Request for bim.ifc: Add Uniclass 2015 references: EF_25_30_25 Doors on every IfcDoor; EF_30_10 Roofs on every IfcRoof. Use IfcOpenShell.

First a look at what the model holds.

```python
import ifcopenshell

model = ifcopenshell.open("bim.ifc")
print(model.schema)
print("classifications:", [c.Name for c in model.by_type("IfcClassification")])
for ifc_class in ("IfcDoor", "IfcRoof", "IfcStair", "IfcWall", "IfcWindow"):
    print(ifc_class, len(model.by_type(ifc_class)))
```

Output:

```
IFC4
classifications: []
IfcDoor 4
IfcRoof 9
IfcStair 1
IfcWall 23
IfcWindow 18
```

```python
import ifcopenshell
import ifcopenshell.api.classification

model = ifcopenshell.open("bim.ifc")

system = ifcopenshell.api.classification.add_classification(model, classification="Uniclass 2015")

codes = {
    "IfcDoor": ("EF_25_30_25", "Doors"),
    "IfcRoof": ("EF_30_10", "Roofs"),
}
for ifc_class, (code, name) in codes.items():
    products = model.by_type(ifc_class)
    ifcopenshell.api.classification.add_reference(
        model, products=products, classification=system, identification=code, name=name
    )
    print(code, len(products))

model.write("bim_edited.ifc")
```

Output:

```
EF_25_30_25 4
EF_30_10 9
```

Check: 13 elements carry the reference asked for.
